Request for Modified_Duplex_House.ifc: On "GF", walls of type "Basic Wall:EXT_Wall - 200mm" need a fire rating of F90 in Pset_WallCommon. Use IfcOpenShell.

First a look at what the model holds.

```python
import ifcopenshell
import ifcopenshell.util.element

model = ifcopenshell.open("Modified_Duplex_House.ifc")
print(model.schema)
storey = next(s for s in model.by_type("IfcBuildingStorey") if s.Name == "GF")
walls = [e for e in ifcopenshell.util.element.get_decomposition(storey) if e.is_a("IfcWall")]
seen = {}
for e in walls:
    element_type = ifcopenshell.util.element.get_type(e)
    key = (element_type.Name if element_type != e and element_type else None, ifcopenshell.util.element.get_pset(e, "Pset_WallCommon", "FireRating"))
    seen[key] = seen.get(key, 0) + 1
for (name, value), count in sorted(seen.items(), key=str):
    print(count, "x", name, "|", value)
```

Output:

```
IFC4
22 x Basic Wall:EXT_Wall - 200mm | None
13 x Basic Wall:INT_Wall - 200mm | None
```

```python
import ifcopenshell
import ifcopenshell.api.pset
import ifcopenshell.util.element

model = ifcopenshell.open("Modified_Duplex_House.ifc")

storey = next(s for s in model.by_type("IfcBuildingStorey") if s.Name == "GF")
walls = [e for e in ifcopenshell.util.element.get_decomposition(storey) if e.is_a("IfcWall")]

count = 0
for e in walls:
    element_type = ifcopenshell.util.element.get_type(e)
    if element_type in (None, e) or element_type.Name != "Basic Wall:EXT_Wall - 200mm":
        continue
    # add_pset returns the element's existing set when there is one.
    pset = ifcopenshell.api.pset.add_pset(model, product=e, name="Pset_WallCommon")
    ifcopenshell.api.pset.edit_pset(model, pset=pset, properties={"FireRating": "F90"})
    count += 1

print(count, "walls updated")

model.write("Modified_Duplex_House_v2.ifc")
```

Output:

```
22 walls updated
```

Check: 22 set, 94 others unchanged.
